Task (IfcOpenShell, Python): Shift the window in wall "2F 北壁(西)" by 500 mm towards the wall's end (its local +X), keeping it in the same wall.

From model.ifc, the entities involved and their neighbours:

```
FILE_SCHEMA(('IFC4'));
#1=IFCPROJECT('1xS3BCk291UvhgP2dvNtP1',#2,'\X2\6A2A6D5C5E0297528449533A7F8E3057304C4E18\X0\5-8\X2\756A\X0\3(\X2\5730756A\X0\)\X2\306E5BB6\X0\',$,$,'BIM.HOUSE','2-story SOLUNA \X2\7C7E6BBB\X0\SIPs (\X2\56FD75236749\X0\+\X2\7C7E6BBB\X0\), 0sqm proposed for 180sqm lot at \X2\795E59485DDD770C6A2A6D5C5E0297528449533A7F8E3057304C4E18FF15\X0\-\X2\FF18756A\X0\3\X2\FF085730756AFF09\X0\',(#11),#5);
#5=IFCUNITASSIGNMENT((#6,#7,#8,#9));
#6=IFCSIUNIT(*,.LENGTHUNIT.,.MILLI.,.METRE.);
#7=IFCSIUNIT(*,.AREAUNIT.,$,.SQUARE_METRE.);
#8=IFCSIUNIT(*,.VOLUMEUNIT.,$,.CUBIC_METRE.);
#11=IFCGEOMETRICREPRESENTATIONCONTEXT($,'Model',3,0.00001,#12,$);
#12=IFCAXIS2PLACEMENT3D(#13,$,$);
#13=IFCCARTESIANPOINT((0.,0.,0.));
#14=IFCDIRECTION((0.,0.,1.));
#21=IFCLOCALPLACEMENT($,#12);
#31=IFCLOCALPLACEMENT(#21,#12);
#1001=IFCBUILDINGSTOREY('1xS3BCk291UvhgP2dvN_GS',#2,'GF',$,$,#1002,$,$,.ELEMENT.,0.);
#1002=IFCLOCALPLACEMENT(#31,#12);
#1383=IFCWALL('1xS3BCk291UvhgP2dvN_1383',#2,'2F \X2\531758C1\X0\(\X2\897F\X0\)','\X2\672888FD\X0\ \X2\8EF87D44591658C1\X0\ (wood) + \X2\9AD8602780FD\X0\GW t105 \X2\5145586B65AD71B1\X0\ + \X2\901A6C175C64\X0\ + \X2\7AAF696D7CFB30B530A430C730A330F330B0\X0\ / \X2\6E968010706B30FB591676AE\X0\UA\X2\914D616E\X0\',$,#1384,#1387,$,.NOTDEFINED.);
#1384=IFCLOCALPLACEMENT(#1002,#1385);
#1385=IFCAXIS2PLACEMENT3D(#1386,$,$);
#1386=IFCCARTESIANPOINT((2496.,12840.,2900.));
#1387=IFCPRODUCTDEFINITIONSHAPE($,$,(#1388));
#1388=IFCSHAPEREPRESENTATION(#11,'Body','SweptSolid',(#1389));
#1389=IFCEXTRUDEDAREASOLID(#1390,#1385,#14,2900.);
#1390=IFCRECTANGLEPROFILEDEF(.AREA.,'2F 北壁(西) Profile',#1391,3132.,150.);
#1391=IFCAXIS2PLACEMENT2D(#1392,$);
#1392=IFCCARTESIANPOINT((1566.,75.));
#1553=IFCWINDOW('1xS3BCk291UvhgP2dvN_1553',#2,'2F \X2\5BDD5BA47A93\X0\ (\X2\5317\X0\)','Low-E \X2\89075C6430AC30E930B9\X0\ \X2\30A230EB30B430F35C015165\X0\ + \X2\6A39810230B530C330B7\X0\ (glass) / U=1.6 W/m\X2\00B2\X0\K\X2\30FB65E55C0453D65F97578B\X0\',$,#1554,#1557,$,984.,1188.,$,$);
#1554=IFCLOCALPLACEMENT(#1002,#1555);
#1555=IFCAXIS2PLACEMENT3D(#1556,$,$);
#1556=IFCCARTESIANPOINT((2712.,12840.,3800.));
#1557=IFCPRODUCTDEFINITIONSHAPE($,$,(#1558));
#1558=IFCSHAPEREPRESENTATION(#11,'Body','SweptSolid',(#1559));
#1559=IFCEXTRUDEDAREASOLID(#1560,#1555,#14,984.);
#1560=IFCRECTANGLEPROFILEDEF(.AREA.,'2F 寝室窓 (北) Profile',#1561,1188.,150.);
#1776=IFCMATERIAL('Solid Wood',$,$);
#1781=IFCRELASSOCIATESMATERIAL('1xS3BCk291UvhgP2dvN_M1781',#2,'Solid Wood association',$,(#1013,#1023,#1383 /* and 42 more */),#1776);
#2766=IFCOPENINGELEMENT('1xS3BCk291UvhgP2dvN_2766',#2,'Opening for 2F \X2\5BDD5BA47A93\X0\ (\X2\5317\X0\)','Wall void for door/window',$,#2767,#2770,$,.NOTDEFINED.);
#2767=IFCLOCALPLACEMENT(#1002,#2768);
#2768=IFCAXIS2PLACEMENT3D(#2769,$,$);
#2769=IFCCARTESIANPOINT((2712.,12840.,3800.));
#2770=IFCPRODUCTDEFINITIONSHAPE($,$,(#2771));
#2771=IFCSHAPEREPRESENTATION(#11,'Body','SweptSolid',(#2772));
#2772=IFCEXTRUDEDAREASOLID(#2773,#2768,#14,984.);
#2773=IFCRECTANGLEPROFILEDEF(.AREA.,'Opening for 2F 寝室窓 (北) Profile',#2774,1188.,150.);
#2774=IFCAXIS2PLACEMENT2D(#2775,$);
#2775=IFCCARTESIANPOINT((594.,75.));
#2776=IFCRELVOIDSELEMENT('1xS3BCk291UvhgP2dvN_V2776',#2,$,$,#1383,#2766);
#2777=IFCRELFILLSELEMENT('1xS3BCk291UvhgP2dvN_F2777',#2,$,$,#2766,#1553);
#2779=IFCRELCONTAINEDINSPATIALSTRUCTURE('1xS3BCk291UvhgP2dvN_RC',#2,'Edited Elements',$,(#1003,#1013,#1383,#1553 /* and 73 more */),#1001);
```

```python
import ifcopenshell
import ifcopenshell.api.geometry
import ifcopenshell.util.placement
import ifcopenshell.util.unit

model = ifcopenshell.open("model.ifc")
unit_scale = ifcopenshell.util.unit.calculate_unit_scale(model)

window = model.by_guid("1xS3BCk291UvhgP2dvN_1553")
opening = window.FillsVoids[0].RelatingOpeningElement
wall = opening.VoidsElements[0].RelatingBuildingElement

wall_matrix = ifcopenshell.util.placement.get_local_placement(wall.ObjectPlacement)
shift = wall_matrix[:3, 0] * 0.5 / unit_scale
before = ifcopenshell.util.placement.get_local_placement(window.ObjectPlacement)[:3, 3].copy()

# The window is not placed relative to its opening, so move both.
for product in (opening, window):
    matrix = ifcopenshell.util.placement.get_local_placement(product.ObjectPlacement)
    matrix[:3, 3] += shift
    ifcopenshell.api.geometry.edit_object_placement(model, product=product, matrix=matrix, is_si=False)

after = ifcopenshell.util.placement.get_local_placement(window.ObjectPlacement)[:3, 3]
print("window moved by", (after - before).round(3) + 0.0)

model.write("model_rev.ifc")
```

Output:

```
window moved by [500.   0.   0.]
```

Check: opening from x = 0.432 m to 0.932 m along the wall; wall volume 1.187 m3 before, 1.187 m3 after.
